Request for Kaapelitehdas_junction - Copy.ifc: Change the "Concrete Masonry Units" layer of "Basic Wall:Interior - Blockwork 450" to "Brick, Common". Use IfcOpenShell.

First a look at what the model holds.

```python
import ifcopenshell
import ifcopenshell.util.element

model = ifcopenshell.open("Kaapelitehdas_junction - Copy.ifc")
print(model.schema)
for layer_set in model.by_type("IfcMaterialLayerSet"):
    if layer_set.LayerSetName == "Basic Wall:Interior - Blockwork 450":
        for layer in layer_set.MaterialLayers:
            print(layer.id(), layer.Material and layer.Material.Name, layer.LayerThickness, sep=" | ")
        print(len(ifcopenshell.util.element.get_elements_by_material(model, layer_set)), "elements and types use it")
print(sorted(m.Name for m in model.by_type("IfcMaterial") if m.Name)[:60])
```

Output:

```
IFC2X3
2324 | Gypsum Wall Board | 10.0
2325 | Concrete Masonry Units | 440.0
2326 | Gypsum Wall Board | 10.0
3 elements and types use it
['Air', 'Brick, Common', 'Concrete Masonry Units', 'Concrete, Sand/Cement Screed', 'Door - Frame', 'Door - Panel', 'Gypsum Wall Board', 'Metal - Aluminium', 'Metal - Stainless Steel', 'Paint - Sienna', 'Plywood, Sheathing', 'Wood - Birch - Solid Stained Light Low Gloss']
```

```python
import ifcopenshell
import ifcopenshell.api.material

model = ifcopenshell.open("Kaapelitehdas_junction - Copy.ifc")

layer_set = next(s for s in model.by_type("IfcMaterialLayerSet") if s.LayerSetName == "Basic Wall:Interior - Blockwork 450")
layer = next(l for l in layer_set.MaterialLayers if l.Material and l.Material.Name == "Concrete Masonry Units")
material = next(m for m in model.by_type("IfcMaterial") if m.Name == "Brick, Common")

# Point this one layer at the other material; renaming the old one would change it everywhere.
ifcopenshell.api.material.edit_layer(model, layer=layer, attributes={}, material=material)

print([l.Material.Name if l.Material else None for l in layer_set.MaterialLayers])

model.write("Kaapelitehdas_junction - Copy_edited.ifc")
```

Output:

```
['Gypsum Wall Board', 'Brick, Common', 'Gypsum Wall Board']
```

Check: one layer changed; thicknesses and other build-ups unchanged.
